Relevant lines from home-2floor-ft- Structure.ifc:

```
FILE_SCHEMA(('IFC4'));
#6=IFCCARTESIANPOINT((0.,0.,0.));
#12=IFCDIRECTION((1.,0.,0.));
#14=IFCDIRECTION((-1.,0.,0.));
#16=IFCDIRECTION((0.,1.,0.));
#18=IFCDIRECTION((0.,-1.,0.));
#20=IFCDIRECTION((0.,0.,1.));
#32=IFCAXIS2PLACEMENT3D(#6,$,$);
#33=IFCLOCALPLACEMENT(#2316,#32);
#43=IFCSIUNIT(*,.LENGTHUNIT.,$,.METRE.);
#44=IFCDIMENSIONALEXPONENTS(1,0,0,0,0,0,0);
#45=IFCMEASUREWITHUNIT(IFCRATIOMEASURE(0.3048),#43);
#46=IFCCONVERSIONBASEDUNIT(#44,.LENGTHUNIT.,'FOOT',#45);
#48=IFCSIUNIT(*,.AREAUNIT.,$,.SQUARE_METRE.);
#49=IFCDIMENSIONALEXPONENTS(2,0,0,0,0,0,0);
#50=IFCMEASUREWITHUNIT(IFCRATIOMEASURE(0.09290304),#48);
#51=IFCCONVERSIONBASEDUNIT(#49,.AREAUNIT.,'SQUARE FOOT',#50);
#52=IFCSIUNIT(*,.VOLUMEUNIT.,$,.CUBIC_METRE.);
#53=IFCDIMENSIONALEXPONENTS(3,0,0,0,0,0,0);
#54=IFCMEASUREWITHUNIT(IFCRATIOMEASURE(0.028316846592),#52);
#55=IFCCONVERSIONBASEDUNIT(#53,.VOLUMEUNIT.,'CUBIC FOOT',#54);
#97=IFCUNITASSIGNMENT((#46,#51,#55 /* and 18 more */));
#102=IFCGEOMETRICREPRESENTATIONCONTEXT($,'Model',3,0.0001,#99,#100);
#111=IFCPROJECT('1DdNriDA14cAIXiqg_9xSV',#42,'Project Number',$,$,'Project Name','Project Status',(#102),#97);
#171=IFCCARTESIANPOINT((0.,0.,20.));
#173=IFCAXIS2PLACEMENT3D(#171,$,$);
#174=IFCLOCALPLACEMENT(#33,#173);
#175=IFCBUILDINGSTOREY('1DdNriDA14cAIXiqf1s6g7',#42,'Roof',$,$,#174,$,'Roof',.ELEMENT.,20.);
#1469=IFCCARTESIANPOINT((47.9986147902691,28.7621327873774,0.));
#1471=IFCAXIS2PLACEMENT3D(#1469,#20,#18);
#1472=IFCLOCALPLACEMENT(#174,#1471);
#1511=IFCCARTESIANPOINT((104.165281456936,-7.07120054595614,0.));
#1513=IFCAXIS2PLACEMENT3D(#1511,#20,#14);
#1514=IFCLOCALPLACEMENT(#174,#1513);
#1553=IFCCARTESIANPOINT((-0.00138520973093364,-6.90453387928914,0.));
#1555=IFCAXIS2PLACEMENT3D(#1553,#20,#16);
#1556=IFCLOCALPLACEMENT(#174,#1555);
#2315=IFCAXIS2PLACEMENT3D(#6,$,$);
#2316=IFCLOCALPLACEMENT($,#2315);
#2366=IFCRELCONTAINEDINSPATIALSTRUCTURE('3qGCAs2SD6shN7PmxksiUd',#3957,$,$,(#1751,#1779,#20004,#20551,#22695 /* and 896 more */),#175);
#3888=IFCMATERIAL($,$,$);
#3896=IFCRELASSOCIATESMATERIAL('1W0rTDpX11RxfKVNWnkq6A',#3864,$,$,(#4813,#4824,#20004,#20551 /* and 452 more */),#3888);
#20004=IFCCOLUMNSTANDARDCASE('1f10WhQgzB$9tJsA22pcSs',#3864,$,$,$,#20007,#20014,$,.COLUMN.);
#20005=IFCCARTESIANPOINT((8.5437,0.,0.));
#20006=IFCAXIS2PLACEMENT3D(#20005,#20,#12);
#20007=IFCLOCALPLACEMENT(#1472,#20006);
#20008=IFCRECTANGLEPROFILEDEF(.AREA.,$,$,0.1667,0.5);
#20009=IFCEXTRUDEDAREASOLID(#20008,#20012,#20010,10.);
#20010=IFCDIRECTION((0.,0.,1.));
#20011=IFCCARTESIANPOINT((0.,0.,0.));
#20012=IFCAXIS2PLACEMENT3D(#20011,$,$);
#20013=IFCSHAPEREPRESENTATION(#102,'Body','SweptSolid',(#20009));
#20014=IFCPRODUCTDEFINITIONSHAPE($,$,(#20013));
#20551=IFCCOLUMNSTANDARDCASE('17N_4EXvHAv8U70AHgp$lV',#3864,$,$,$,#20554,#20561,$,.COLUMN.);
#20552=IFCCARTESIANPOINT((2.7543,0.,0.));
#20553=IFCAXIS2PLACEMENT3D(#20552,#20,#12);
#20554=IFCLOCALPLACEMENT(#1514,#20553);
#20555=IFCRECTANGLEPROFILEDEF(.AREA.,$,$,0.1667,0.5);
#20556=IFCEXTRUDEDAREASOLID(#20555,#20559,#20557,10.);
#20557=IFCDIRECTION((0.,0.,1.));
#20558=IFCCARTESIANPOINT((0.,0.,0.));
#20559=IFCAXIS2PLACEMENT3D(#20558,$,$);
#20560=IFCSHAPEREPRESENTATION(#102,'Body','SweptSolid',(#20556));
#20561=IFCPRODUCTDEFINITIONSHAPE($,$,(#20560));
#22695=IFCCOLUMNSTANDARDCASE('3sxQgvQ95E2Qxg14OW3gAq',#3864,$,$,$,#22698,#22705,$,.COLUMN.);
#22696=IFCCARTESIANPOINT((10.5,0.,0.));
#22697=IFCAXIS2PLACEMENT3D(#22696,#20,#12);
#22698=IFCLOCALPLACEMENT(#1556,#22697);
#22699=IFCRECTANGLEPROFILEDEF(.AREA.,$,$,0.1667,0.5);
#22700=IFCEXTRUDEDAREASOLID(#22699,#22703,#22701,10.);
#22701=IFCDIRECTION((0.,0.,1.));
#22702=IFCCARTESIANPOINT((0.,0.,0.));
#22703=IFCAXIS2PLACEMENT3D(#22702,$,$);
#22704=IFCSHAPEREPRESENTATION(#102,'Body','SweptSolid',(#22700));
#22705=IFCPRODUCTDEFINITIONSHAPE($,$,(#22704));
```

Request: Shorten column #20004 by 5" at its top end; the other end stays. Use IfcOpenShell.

```python
import ifcopenshell
import ifcopenshell.util.unit

model = ifcopenshell.open("home-2floor-ft- Structure.ifc")
unit_scale = ifcopenshell.util.unit.calculate_unit_scale(model)

member = model.by_guid("1f10WhQgzB$9tJsA22pcSs")
change = -5 * 0.0254 / unit_scale

# The extrusion runs towards the end named, so only its depth changes.
body = next(r for r in member.Representation.Representations if r.RepresentationIdentifier == "Body")
solid = body.Items[0]
old_length = solid.Depth
solid.Depth += change

print(f"length {old_length:g} -> {solid.Depth:g}")

model.write("home-2floor-ft- Structure_v2.ifc")
```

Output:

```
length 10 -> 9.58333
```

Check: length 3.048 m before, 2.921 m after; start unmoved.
